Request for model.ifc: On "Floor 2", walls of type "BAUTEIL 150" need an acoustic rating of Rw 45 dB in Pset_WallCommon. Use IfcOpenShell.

First a look at what the model holds.

```python
import ifcopenshell
import ifcopenshell.util.element

model = ifcopenshell.open("model.ifc")
print(model.schema)
storey = next(s for s in model.by_type("IfcBuildingStorey") if s.Name == "Floor 2")
walls = [e for e in ifcopenshell.util.element.get_decomposition(storey) if e.is_a("IfcWall")]
seen = {}
for e in walls:
    element_type = ifcopenshell.util.element.get_type(e)
    key = (element_type.Name if element_type != e and element_type else None, ifcopenshell.util.element.get_pset(e, "Pset_WallCommon", "AcousticRating"))
    seen[key] = seen.get(key, 0) + 1
for (name, value), count in sorted(seen.items(), key=str):
    print(count, "x", name, "|", value)
```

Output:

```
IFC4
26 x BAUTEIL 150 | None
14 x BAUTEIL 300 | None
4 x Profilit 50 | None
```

```python
import ifcopenshell
import ifcopenshell.api.pset
import ifcopenshell.util.element

model = ifcopenshell.open("model.ifc")

storey = next(s for s in model.by_type("IfcBuildingStorey") if s.Name == "Floor 2")
walls = [e for e in ifcopenshell.util.element.get_decomposition(storey) if e.is_a("IfcWall")]

count = 0
for e in walls:
    element_type = ifcopenshell.util.element.get_type(e)
    if element_type in (None, e) or element_type.Name != "BAUTEIL 150":
        continue
    # add_pset returns the element's existing set when there is one.
    pset = ifcopenshell.api.pset.add_pset(model, product=e, name="Pset_WallCommon")
    ifcopenshell.api.pset.edit_pset(model, pset=pset, properties={"AcousticRating": "Rw 45 dB"})
    count += 1

print(count, "walls updated")

model.write("model_edited.ifc")
```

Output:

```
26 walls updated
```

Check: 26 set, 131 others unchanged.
